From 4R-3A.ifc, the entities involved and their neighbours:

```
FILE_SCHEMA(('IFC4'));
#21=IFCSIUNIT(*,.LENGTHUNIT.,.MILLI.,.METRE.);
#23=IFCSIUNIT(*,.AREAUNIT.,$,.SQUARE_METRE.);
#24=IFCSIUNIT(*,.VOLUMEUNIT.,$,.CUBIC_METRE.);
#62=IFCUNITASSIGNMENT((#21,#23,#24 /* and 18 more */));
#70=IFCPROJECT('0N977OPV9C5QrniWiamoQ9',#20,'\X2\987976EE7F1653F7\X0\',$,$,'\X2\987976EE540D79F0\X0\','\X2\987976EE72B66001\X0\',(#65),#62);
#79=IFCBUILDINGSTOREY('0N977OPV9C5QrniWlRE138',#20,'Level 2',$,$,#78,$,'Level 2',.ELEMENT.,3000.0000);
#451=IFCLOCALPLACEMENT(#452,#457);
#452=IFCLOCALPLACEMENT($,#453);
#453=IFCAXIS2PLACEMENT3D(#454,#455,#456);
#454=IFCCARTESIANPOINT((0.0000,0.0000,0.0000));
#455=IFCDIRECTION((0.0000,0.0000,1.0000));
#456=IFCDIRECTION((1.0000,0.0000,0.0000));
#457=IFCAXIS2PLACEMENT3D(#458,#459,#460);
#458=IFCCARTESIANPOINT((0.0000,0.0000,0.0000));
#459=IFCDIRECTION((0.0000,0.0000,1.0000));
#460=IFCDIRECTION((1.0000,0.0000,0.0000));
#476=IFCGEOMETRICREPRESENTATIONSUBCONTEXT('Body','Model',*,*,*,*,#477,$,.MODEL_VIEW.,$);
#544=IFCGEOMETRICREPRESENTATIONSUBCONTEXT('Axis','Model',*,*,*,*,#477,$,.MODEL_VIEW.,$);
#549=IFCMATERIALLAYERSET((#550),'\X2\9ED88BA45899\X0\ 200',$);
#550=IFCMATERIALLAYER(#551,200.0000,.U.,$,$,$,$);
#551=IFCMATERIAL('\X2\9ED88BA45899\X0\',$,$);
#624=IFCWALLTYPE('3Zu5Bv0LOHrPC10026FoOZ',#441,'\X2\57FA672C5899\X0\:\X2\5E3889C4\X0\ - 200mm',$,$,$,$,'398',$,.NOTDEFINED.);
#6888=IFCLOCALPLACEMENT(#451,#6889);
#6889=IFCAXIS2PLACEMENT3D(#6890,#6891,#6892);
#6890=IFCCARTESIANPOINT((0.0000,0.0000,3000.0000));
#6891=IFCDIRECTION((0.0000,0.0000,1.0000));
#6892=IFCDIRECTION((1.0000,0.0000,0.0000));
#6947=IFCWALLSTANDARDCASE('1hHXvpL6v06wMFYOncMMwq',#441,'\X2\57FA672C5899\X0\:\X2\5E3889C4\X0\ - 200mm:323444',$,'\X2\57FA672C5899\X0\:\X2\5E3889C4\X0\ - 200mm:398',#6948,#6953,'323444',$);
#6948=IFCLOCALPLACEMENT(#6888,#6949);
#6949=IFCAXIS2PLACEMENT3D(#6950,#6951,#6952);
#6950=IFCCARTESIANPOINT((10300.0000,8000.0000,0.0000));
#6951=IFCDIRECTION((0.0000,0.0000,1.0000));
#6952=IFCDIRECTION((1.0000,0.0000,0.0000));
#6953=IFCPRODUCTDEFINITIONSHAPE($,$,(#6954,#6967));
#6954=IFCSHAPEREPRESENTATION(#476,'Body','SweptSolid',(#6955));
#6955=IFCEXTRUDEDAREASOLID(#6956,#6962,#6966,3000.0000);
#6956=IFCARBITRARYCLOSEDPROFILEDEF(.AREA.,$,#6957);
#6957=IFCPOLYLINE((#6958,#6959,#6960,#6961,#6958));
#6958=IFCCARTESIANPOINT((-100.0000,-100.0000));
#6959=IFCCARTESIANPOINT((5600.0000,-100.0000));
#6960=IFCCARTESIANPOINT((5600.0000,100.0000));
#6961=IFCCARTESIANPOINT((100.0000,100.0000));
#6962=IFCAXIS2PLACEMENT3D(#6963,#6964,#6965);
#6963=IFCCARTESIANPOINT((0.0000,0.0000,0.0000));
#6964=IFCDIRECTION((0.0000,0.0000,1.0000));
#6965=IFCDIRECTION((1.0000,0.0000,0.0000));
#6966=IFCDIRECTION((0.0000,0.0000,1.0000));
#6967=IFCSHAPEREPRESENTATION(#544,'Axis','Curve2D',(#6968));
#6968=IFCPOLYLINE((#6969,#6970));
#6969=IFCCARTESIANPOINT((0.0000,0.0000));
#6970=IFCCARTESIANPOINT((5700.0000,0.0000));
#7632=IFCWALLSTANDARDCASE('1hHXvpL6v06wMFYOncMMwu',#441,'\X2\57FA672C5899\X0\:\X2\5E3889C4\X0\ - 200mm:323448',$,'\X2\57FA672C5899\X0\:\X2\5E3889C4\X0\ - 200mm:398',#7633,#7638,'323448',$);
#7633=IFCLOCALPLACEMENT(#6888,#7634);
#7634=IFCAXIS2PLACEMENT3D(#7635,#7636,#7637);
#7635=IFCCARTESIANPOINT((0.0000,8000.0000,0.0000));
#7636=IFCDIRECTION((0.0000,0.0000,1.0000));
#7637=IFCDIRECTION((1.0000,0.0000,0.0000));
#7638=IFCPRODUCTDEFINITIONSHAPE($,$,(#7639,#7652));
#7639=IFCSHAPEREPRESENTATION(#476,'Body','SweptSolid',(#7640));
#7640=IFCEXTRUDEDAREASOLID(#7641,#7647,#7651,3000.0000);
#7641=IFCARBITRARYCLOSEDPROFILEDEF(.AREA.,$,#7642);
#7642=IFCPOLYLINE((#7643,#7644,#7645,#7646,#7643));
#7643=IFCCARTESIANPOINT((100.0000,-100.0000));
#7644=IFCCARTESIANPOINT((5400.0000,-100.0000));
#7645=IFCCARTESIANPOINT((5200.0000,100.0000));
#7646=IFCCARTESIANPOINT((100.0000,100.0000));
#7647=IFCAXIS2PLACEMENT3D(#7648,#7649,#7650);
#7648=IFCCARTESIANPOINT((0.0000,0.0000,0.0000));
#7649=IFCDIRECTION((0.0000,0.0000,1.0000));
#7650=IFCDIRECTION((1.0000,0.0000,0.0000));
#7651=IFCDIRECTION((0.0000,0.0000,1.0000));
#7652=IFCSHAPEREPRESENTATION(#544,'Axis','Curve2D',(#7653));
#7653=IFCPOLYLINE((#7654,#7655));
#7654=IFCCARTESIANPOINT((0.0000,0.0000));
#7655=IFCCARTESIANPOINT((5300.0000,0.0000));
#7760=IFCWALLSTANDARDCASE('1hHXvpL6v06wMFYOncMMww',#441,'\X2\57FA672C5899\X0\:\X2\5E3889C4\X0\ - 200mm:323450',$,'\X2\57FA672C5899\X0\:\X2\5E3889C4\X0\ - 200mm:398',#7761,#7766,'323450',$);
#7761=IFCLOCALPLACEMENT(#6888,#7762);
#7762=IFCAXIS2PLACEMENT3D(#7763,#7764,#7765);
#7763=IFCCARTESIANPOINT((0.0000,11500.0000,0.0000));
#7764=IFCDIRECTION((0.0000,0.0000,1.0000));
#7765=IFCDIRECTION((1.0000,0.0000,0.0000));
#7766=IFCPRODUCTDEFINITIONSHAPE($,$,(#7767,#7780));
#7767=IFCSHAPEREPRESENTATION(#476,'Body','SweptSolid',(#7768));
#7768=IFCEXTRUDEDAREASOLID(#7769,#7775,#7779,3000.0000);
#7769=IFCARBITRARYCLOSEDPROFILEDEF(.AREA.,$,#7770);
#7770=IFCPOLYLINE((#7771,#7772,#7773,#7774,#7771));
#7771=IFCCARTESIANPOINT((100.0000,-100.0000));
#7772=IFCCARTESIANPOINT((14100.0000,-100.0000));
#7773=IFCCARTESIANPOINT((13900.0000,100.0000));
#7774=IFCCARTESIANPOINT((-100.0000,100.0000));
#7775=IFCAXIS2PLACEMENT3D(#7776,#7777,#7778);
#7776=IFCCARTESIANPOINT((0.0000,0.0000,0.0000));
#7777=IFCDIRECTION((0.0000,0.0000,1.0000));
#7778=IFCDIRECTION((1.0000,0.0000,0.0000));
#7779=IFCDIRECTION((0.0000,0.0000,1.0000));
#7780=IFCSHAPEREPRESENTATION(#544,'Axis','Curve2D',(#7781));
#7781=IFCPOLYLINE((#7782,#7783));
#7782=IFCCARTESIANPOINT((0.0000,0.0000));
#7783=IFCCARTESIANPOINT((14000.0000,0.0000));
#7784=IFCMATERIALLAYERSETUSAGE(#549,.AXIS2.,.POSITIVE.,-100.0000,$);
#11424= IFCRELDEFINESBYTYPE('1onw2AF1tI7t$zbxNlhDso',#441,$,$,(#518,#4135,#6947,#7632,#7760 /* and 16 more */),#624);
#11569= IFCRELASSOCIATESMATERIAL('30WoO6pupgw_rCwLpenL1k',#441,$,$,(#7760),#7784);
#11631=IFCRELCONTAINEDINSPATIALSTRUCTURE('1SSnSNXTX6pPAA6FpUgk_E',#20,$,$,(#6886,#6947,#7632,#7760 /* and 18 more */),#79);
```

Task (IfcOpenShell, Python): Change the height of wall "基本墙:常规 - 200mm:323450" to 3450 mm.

```python
import ifcopenshell
import ifcopenshell.geom
import ifcopenshell.util.representation
import ifcopenshell.util.shape
import ifcopenshell.util.unit

model = ifcopenshell.open("4R-3A.ifc")
unit_scale = ifcopenshell.util.unit.calculate_unit_scale(model)
settings = ifcopenshell.geom.settings()


def volume(element):
    """Net volume in cubic metres, openings subtracted."""
    shape = ifcopenshell.geom.create_shape(settings, element)
    return ifcopenshell.util.shape.get_volume(shape.geometry)


wall = model.by_guid("1hHXvpL6v06wMFYOncMMww")
before = volume(wall)

body = ifcopenshell.util.representation.get_representation(wall, "Model", "Body")
solid = body.Items[0]
old_height = solid.Depth
solid.Depth = 3.45 / unit_scale
after = volume(wall)

print(f"height {old_height:g} -> {solid.Depth:g}, volume {before:.3f} -> {after:.3f} m3")

model.write("4R-3A_edited.ifc")
```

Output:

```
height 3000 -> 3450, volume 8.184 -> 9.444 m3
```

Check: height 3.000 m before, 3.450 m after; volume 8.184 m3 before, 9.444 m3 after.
